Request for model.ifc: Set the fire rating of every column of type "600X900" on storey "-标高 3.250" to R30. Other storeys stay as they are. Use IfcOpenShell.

First a look at what the model holds.

```python
import ifcopenshell
import ifcopenshell.util.element

model = ifcopenshell.open("model.ifc")
print(model.schema)
storey = next(s for s in model.by_type("IfcBuildingStorey") if s.Name == "-标高 3.250")
columns = [e for e in ifcopenshell.util.element.get_decomposition(storey) if e.is_a("IfcColumn")]
seen = {}
for e in columns:
    element_type = ifcopenshell.util.element.get_type(e)
    key = (element_type.Name if element_type != e and element_type else None, ifcopenshell.util.element.get_pset(e, "Pset_ColumnCommon", "FireRating"))
    seen[key] = seen.get(key, 0) + 1
for (name, value), count in sorted(seen.items(), key=str):
    print(count, "x", name, "|", value)
```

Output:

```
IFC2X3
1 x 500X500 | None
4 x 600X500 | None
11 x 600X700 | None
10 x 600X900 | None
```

```python
import ifcopenshell
import ifcopenshell.api.pset
import ifcopenshell.util.element

model = ifcopenshell.open("model.ifc")

storey = next(s for s in model.by_type("IfcBuildingStorey") if s.Name == "-标高 3.250")
columns = [e for e in ifcopenshell.util.element.get_decomposition(storey) if e.is_a("IfcColumn")]

count = 0
for e in columns:
    element_type = ifcopenshell.util.element.get_type(e)
    if element_type in (None, e) or element_type.Name != "600X900":
        continue
    # add_pset returns the element's existing set when there is one.
    pset = ifcopenshell.api.pset.add_pset(model, product=e, name="Pset_ColumnCommon")
    ifcopenshell.api.pset.edit_pset(model, pset=pset, properties={"FireRating": "R30"})
    count += 1

print(count, "columns updated")

model.write("model_edited.ifc")
```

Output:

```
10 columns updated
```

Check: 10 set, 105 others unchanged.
